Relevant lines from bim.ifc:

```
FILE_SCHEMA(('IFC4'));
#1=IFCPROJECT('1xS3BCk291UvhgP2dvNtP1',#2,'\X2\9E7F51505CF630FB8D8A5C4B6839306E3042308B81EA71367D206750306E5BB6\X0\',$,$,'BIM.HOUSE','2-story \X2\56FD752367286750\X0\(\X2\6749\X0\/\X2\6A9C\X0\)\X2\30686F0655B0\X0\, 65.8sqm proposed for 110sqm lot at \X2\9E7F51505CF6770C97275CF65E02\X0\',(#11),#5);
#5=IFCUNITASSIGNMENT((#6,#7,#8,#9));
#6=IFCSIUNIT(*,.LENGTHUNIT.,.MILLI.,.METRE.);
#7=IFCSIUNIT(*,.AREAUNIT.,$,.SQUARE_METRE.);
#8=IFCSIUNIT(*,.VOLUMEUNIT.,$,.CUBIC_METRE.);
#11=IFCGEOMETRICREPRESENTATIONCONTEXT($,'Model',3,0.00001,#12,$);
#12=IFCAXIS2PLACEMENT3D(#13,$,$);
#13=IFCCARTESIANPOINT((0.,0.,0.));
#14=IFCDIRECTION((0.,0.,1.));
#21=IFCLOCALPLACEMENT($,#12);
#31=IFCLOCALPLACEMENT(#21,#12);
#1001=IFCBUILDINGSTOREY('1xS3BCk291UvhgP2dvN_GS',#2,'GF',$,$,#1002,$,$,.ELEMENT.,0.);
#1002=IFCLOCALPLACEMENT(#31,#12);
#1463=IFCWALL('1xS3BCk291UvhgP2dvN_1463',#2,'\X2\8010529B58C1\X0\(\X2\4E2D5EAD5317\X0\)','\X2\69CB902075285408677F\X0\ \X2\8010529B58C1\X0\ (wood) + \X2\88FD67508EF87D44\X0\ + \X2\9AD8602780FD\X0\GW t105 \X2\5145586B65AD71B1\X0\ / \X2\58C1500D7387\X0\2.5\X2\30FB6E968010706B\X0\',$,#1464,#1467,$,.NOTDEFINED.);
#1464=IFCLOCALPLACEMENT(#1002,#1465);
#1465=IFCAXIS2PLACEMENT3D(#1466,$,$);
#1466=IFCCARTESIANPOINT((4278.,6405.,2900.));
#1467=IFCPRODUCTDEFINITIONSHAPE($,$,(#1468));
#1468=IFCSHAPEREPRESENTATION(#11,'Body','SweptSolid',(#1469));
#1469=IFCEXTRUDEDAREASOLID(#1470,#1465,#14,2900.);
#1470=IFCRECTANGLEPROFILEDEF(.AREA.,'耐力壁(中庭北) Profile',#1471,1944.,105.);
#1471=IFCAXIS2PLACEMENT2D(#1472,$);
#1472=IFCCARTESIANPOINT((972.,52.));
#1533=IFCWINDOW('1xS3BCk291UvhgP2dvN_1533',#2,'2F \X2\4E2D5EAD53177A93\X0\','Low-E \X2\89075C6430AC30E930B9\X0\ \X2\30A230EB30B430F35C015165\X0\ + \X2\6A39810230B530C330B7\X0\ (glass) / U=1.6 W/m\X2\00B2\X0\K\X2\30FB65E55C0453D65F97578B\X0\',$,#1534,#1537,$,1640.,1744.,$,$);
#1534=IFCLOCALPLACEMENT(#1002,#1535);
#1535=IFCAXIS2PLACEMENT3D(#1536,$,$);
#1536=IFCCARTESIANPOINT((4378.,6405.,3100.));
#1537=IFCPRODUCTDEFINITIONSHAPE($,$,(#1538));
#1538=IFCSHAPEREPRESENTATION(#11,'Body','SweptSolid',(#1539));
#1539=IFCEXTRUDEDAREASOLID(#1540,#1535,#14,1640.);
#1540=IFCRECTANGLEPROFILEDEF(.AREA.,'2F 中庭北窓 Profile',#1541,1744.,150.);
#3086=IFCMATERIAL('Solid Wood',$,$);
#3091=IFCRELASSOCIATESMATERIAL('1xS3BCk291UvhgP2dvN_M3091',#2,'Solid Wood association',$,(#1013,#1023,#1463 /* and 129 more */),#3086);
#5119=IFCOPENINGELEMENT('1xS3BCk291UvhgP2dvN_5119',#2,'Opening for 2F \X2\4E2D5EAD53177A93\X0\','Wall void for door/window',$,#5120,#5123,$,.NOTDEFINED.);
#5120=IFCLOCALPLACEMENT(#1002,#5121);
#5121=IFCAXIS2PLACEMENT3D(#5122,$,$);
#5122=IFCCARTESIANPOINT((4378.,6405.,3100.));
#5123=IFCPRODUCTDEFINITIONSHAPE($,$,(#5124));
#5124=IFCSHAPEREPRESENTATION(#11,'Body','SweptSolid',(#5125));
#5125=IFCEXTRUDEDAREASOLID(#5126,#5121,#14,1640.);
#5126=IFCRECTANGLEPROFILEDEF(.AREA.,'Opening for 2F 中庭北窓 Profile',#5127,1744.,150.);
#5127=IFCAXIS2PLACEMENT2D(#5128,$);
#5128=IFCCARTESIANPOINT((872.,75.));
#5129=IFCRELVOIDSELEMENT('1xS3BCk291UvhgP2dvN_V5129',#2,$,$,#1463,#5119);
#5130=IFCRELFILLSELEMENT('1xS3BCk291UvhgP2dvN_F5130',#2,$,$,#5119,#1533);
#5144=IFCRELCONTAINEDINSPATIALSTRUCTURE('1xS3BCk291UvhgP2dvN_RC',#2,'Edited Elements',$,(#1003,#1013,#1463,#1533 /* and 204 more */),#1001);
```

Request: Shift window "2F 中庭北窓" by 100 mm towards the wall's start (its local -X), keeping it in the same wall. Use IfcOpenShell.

```python
import ifcopenshell
import ifcopenshell.api.geometry
import ifcopenshell.util.placement

model = ifcopenshell.open("bim.ifc")

window = model.by_id(1533)
opening = window.FillsVoids[0].RelatingOpeningElement
wall = opening.VoidsElements[0].RelatingBuildingElement

wall_matrix = ifcopenshell.util.placement.get_local_placement(wall.ObjectPlacement)
shift = wall_matrix[:3, 0] * -100.0
before = ifcopenshell.util.placement.get_local_placement(window.ObjectPlacement)[:3, 3].copy()

# The window is not placed relative to its opening, so move both.
for product in (opening, window):
    matrix = ifcopenshell.util.placement.get_local_placement(product.ObjectPlacement)
    matrix[:3, 3] += shift
    ifcopenshell.api.geometry.edit_object_placement(model, product=product, matrix=matrix, is_si=False)

after = ifcopenshell.util.placement.get_local_placement(window.ObjectPlacement)[:3, 3]
print("window moved by", (after - before).round(3) + 0.0)

model.write("bim_edited.ifc")
```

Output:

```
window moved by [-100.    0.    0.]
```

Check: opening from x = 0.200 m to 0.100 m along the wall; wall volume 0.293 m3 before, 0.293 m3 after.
